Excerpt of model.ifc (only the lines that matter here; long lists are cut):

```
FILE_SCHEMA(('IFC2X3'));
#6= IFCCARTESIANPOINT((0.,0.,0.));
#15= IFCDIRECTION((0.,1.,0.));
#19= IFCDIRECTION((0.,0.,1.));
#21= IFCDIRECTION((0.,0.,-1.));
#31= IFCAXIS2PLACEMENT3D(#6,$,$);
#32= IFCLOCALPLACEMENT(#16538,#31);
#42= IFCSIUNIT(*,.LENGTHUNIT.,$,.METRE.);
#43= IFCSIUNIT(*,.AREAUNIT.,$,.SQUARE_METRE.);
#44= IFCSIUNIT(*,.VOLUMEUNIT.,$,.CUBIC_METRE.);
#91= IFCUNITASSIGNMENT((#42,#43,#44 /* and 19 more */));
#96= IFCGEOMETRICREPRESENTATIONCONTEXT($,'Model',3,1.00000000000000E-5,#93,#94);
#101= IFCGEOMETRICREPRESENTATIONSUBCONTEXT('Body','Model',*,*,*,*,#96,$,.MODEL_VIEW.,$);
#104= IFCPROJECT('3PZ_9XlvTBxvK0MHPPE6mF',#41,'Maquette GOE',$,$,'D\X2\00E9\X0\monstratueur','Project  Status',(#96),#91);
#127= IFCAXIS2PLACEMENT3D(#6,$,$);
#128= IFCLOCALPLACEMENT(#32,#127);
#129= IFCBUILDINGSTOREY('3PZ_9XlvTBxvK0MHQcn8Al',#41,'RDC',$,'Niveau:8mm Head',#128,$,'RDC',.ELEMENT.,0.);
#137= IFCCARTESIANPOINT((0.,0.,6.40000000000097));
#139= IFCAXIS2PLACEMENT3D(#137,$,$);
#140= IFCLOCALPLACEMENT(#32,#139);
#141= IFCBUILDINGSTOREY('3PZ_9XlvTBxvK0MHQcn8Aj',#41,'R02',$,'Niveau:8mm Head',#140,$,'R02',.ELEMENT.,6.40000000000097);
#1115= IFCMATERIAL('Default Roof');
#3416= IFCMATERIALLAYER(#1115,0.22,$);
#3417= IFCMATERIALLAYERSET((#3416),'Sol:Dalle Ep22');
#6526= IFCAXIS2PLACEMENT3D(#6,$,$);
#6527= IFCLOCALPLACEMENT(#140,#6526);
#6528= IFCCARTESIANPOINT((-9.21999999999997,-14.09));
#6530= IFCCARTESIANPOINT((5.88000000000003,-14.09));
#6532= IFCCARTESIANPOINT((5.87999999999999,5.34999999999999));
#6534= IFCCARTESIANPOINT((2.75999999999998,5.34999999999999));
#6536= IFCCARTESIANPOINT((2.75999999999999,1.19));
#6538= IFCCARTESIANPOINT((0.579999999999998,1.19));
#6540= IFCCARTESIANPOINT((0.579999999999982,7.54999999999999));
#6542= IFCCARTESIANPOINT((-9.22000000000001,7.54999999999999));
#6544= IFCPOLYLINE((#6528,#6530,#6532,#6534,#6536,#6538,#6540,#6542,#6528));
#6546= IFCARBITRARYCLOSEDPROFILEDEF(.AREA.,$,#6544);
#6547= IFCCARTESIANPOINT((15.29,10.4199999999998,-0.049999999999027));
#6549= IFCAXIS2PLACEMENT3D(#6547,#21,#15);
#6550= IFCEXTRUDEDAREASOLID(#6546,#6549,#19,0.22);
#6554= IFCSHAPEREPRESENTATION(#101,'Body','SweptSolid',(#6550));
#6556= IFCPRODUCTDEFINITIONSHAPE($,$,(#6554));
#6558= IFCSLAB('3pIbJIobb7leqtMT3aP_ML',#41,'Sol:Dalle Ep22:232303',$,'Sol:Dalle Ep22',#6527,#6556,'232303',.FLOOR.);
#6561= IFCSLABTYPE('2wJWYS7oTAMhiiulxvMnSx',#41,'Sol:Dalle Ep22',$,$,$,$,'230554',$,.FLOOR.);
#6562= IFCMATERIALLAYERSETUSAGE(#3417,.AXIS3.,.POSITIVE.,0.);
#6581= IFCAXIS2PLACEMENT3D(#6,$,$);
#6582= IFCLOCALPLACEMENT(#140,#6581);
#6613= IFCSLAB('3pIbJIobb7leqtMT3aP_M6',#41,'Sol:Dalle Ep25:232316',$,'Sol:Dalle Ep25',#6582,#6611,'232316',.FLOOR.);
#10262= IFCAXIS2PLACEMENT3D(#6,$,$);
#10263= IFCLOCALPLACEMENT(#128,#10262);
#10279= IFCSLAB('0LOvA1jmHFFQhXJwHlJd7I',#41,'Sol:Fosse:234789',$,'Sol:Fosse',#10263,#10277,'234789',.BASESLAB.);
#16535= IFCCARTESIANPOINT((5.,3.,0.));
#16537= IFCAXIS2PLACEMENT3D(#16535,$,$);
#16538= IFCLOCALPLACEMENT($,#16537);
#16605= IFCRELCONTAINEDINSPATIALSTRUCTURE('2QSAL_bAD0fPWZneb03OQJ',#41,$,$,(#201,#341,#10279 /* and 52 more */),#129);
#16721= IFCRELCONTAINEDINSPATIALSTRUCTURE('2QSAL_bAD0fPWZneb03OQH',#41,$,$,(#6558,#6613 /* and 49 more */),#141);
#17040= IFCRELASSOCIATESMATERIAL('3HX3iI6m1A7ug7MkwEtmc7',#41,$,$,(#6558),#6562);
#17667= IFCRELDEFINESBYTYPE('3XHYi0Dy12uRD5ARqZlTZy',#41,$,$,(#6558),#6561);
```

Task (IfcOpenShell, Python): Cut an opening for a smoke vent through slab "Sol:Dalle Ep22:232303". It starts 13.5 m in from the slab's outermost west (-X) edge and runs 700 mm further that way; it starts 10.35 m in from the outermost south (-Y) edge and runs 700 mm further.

```python
import numpy as np
import ifcopenshell
import ifcopenshell.api.feature
import ifcopenshell.api.geometry
import ifcopenshell.api.root
import ifcopenshell.geom
import ifcopenshell.util.placement
import ifcopenshell.util.representation
import ifcopenshell.util.shape
import ifcopenshell.util.unit

model = ifcopenshell.open("model.ifc")
unit_scale = ifcopenshell.util.unit.calculate_unit_scale(model)
settings = ifcopenshell.geom.settings()


def volume(element):
    """Net volume in cubic metres, openings subtracted."""
    shape = ifcopenshell.geom.create_shape(settings, element)
    return ifcopenshell.util.shape.get_volume(shape.geometry)


slab = model.by_guid("3pIbJIobb7leqtMT3aP_ML")
before = volume(slab)

# Extent in the slab's own axes, in metres. The edges named are its -X and -Y sides.
slab_shape = ifcopenshell.geom.create_shape(settings, slab)
vertices = ifcopenshell.util.shape.get_vertices(slab_shape.geometry)
x_min, y_min, bottom = vertices.min(axis=0)
top = vertices[:, 2].max()

opening = ifcopenshell.api.root.create_entity(model, ifc_class="IfcOpeningElement", name="Smoke vent opening")
context = ifcopenshell.util.representation.get_context(model, "Model", "Body", "MODEL_VIEW")
width, depth = 0.7, 0.7
outline = [(0.0, 0.0), (width, 0.0), (width, depth), (0.0, depth), (0.0, 0.0)]
# Overshoot both faces by 50 mm so the cut is clean.
shape = ifcopenshell.api.geometry.add_slab_representation(
    model, context=context, depth=top - bottom + 0.1, polyline=outline
)
ifcopenshell.api.geometry.assign_representation(model, product=opening, representation=shape)

matrix = ifcopenshell.util.placement.get_local_placement(slab.ObjectPlacement)
matrix[:, 3] = matrix @ np.append(np.array([x_min + 13.5, y_min + 10.35, bottom - 0.05]) / unit_scale, 1.0)
ifcopenshell.api.geometry.edit_object_placement(model, product=opening, matrix=matrix, is_si=False)
ifcopenshell.api.feature.add_feature(model, feature=opening, element=slab)

after = volume(slab)

print(f"slab volume {before:.3f} -> {after:.3f} m3")

model.write("model_edited.ifc")
```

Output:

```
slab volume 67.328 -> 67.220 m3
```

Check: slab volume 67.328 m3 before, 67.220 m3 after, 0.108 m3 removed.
